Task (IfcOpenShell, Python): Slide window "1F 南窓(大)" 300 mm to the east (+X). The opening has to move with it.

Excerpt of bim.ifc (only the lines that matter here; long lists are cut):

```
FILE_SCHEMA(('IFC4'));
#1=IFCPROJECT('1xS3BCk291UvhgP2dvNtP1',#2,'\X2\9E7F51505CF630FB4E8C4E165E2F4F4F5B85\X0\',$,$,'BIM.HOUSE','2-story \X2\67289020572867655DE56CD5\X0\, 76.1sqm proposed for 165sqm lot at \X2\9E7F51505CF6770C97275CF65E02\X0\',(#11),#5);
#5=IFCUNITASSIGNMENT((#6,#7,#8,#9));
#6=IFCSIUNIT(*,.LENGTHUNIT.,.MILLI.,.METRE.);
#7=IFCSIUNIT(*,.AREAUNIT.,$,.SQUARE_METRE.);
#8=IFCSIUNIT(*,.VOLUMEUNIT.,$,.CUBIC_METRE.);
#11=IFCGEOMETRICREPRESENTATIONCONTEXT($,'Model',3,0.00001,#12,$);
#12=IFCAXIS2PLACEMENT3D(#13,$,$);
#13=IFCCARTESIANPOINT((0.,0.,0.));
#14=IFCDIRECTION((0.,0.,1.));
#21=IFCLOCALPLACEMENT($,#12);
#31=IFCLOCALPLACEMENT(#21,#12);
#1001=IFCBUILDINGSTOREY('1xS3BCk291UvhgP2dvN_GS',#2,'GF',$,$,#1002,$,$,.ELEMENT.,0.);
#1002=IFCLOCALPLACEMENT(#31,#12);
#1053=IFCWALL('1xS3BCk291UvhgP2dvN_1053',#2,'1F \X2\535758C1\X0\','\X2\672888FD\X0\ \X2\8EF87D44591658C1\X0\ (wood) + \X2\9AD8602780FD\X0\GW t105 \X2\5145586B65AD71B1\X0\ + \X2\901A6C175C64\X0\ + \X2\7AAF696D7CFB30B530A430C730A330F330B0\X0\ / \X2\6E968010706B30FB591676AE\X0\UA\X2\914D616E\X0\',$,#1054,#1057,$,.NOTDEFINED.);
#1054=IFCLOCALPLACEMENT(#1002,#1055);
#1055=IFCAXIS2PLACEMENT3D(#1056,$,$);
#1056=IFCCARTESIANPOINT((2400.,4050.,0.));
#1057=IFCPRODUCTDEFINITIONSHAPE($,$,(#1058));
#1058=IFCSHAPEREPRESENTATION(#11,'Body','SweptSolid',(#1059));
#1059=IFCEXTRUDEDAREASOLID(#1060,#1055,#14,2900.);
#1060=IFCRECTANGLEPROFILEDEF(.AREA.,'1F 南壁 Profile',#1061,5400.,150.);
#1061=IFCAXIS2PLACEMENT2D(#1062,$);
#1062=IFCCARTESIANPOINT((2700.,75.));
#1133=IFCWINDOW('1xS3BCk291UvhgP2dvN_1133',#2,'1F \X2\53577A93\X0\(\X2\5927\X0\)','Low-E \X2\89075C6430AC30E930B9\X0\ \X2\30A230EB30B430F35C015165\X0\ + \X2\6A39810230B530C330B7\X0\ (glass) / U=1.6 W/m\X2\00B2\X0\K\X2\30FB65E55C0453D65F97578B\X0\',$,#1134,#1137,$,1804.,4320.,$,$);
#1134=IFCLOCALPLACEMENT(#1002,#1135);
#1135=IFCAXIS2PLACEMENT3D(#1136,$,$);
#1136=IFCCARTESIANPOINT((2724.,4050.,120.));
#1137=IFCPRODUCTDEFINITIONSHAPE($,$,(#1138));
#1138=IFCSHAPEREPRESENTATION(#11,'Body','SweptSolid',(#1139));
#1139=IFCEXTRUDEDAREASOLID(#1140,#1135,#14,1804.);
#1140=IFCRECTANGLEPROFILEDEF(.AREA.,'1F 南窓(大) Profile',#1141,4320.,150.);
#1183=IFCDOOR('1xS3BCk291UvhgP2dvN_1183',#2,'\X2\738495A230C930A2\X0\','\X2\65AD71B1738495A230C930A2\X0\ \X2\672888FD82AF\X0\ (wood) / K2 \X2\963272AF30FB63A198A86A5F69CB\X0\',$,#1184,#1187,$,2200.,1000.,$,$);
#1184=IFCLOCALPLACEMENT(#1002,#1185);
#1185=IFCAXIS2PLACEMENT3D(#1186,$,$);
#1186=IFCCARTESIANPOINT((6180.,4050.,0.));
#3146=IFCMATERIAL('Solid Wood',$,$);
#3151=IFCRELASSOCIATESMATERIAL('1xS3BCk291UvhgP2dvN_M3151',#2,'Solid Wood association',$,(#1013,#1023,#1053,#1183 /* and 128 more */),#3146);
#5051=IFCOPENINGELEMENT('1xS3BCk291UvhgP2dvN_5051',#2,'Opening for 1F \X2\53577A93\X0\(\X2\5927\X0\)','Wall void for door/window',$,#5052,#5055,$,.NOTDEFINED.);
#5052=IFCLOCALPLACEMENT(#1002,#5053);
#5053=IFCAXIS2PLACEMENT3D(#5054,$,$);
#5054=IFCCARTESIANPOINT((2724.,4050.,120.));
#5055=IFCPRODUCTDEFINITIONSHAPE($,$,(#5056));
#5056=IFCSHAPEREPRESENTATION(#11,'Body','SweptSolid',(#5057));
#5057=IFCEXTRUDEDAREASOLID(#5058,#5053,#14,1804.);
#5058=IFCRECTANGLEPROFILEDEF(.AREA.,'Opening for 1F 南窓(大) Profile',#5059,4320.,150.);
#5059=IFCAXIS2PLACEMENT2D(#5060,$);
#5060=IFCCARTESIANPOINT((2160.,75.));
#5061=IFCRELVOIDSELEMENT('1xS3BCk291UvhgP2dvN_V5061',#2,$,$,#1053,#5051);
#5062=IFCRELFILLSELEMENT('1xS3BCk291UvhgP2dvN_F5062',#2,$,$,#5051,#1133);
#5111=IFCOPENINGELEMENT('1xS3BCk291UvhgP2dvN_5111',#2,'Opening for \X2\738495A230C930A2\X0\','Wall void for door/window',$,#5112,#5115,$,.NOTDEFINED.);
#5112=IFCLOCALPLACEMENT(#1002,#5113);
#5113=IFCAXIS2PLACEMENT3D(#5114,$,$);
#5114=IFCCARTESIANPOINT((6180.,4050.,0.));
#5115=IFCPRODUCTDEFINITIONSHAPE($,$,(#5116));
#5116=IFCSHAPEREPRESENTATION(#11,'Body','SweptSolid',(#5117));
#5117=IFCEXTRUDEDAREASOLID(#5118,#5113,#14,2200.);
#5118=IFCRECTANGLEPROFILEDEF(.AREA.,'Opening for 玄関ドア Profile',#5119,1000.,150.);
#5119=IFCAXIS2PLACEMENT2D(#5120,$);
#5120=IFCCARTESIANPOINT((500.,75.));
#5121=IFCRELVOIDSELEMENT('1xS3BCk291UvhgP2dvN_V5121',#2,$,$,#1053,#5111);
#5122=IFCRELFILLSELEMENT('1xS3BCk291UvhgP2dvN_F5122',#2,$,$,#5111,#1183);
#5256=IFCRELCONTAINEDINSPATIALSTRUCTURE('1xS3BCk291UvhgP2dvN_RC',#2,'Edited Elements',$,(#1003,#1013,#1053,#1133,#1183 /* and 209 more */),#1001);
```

```python
import ifcopenshell
import ifcopenshell.api.geometry
import ifcopenshell.util.placement

model = ifcopenshell.open("bim.ifc")

window = model.by_guid("1xS3BCk291UvhgP2dvN_1133")
opening = window.FillsVoids[0].RelatingOpeningElement
wall = opening.VoidsElements[0].RelatingBuildingElement

wall_matrix = ifcopenshell.util.placement.get_local_placement(wall.ObjectPlacement)
shift = wall_matrix[:3, 0] * 300.0
before = ifcopenshell.util.placement.get_local_placement(window.ObjectPlacement)[:3, 3].copy()

# The window is not placed relative to its opening, so move both.
for product in (opening, window):
    matrix = ifcopenshell.util.placement.get_local_placement(product.ObjectPlacement)
    matrix[:3, 3] += shift
    ifcopenshell.api.geometry.edit_object_placement(model, product=product, matrix=matrix, is_si=False)

after = ifcopenshell.util.placement.get_local_placement(window.ObjectPlacement)[:3, 3]
print("window moved by", (after - before).round(3) + 0.0)

model.write("bim_v2.ifc")
```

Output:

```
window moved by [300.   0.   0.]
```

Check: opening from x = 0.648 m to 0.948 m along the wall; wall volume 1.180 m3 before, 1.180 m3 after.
